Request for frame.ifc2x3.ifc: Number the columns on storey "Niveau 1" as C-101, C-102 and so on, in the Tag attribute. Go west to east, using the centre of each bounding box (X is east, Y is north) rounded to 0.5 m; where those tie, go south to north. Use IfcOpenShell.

First a look at what the model holds.

```python
import ifcopenshell
import ifcopenshell.util.element
import ifcopenshell.util.placement

model = ifcopenshell.open("frame.ifc2x3.ifc")
print(model.schema)
storey = next(s for s in model.by_type("IfcBuildingStorey") if s.Name == "Niveau 1")
columns = [e for e in ifcopenshell.util.element.get_decomposition(storey) if e.is_a("IfcColumn")]
for e in sorted(columns, key=lambda e: e.id()):
    origin = ifcopenshell.util.placement.get_local_placement(e.ObjectPlacement)[:3, 3]
    print(e.id(), e.Tag, e.Name, origin.round(2) + 0.0, sep=" | ")
```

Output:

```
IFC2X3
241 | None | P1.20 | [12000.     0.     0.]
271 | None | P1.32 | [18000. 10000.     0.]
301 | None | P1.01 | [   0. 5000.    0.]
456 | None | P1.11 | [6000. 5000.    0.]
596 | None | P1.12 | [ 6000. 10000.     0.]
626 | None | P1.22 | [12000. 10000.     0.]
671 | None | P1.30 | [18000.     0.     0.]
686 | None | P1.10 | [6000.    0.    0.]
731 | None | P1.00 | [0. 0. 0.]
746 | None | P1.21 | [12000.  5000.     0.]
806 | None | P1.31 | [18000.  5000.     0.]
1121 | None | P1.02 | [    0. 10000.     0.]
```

```python
import ifcopenshell
import ifcopenshell.geom
import ifcopenshell.util.element
import ifcopenshell.util.shape

model = ifcopenshell.open("frame.ifc2x3.ifc")
settings = ifcopenshell.geom.settings()
settings.set("use-world-coords", True)


def centre(element):
    shape = ifcopenshell.geom.create_shape(settings, element)
    return ifcopenshell.util.shape.get_bbox_centroid(shape.geometry)


storey = next(s for s in model.by_type("IfcBuildingStorey") if s.Name == "Niveau 1")
columns = [e for e in ifcopenshell.util.element.get_decomposition(storey) if e.is_a("IfcColumn")]

# Insertion points can sit at a corner or the storey origin, so sort by the geometry (in metres).
centres = {e: centre(e) for e in columns}
columns.sort(key=lambda e: (round(centres[e][0] / 0.5), centres[e][1]))

for i, e in enumerate(columns, start=1):
    number = f"C-1{i:02d}"
    e.Tag = number
    print(e.id(), number)

model.write("frame.ifc2x3_v2.ifc")
```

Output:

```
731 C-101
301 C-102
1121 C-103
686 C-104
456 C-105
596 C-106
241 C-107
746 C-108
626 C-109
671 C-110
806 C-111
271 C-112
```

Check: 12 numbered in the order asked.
